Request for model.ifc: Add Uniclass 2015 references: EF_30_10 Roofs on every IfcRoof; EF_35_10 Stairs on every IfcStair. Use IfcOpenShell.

First a look at what the model holds.

```python
import ifcopenshell

model = ifcopenshell.open("model.ifc")
print(model.schema)
print("classifications:", [c.Name for c in model.by_type("IfcClassification")])
for ifc_class in ("IfcDoor", "IfcRoof", "IfcStair", "IfcWall", "IfcWindow"):
    print(ifc_class, len(model.by_type(ifc_class)))
```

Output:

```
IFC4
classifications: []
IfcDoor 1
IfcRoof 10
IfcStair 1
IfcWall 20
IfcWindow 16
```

```python
import ifcopenshell
import ifcopenshell.api.classification

model = ifcopenshell.open("model.ifc")

system = ifcopenshell.api.classification.add_classification(model, classification="Uniclass 2015")

codes = {
    "IfcRoof": ("EF_30_10", "Roofs"),
    "IfcStair": ("EF_35_10", "Stairs"),
}
for ifc_class, (code, name) in codes.items():
    products = model.by_type(ifc_class)
    ifcopenshell.api.classification.add_reference(
        model, products=products, classification=system, identification=code, name=name
    )
    print(code, len(products))

model.write("model_rev.ifc")
```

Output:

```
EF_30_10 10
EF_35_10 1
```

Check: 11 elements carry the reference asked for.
